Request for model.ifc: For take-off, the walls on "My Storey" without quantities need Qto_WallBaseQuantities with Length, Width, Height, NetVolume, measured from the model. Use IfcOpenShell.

First a look at what the model holds.

```python
import ifcopenshell
import ifcopenshell.util.element
import ifcopenshell.util.unit

model = ifcopenshell.open("model.ifc")
print(model.schema)
for unit_type in ("LENGTHUNIT", "AREAUNIT", "VOLUMEUNIT"):
    print(unit_type, ifcopenshell.util.unit.calculate_unit_scale(model, unit_type))
storey = next(s for s in model.by_type("IfcBuildingStorey") if s.Name == "My Storey")
walls = [e for e in ifcopenshell.util.element.get_decomposition(storey) if e.is_a("IfcWall")]
for e in sorted(walls, key=lambda e: e.id()):
    print(e.id(), e.is_a(), e.Name, list(ifcopenshell.util.element.get_psets(e, qtos_only=True)), sep=" | ")
```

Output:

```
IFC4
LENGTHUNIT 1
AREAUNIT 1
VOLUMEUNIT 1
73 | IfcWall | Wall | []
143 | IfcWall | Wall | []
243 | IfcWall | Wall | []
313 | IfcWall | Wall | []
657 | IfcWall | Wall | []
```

```python
import ifcopenshell
import ifcopenshell.api.pset
import ifcopenshell.geom
import ifcopenshell.util.element
import ifcopenshell.util.shape
import ifcopenshell.util.unit

model = ifcopenshell.open("model.ifc")
unit_scale = ifcopenshell.util.unit.calculate_unit_scale(model)
volume_scale = ifcopenshell.util.unit.calculate_unit_scale(model, "VOLUMEUNIT")
settings = ifcopenshell.geom.settings()

storey = next(s for s in model.by_type("IfcBuildingStorey") if s.Name == "My Storey")
walls = [e for e in ifcopenshell.util.element.get_decomposition(storey) if e.is_a("IfcWall")]

for e in sorted(walls, key=lambda e: e.id()):
    if ifcopenshell.util.element.get_psets(e, qtos_only=True, should_inherit=False):
        continue
    # Geometry comes back in metres, in the element's own axes.
    shape = ifcopenshell.geom.create_shape(settings, e)
    values = {
        "Length": ifcopenshell.util.shape.get_x(shape.geometry) / unit_scale,
        "Width": ifcopenshell.util.shape.get_y(shape.geometry) / unit_scale,
        "Height": ifcopenshell.util.shape.get_z(shape.geometry) / unit_scale,
        "NetVolume": ifcopenshell.util.shape.get_volume(shape.geometry) / volume_scale,
    }
    qto = ifcopenshell.api.pset.add_qto(model, product=e, name="Qto_WallBaseQuantities")
    ifcopenshell.api.pset.edit_qto(model, qto=qto, properties=values)
    print(e.id(), {k: round(v, 3) for k, v in values.items()})

model.write("model_edited.ifc")
```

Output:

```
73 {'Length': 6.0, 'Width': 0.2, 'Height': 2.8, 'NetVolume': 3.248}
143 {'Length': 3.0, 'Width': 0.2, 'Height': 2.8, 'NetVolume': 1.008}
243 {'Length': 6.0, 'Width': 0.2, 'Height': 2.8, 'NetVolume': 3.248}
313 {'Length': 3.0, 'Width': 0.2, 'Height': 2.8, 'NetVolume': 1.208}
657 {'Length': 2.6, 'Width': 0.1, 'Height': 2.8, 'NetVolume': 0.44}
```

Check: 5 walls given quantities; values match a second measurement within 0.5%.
